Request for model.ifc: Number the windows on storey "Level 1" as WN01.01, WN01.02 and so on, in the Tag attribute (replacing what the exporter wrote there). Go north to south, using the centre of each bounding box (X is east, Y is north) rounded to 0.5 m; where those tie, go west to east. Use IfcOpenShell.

First a look at what the model holds.

```python
import ifcopenshell
import ifcopenshell.util.element
import ifcopenshell.util.placement

model = ifcopenshell.open("model.ifc")
print(model.schema)
storey = next(s for s in model.by_type("IfcBuildingStorey") if s.Name == "Level 1")
windows = [e for e in ifcopenshell.util.element.get_decomposition(storey) if e.is_a("IfcWindow")]
for e in sorted(windows, key=lambda e: e.id()):
    origin = ifcopenshell.util.placement.get_local_placement(e.ObjectPlacement)[:3, 3]
    print(e.id(), e.Tag, e.Name, origin.round(2) + 0.0, sep=" | ")
```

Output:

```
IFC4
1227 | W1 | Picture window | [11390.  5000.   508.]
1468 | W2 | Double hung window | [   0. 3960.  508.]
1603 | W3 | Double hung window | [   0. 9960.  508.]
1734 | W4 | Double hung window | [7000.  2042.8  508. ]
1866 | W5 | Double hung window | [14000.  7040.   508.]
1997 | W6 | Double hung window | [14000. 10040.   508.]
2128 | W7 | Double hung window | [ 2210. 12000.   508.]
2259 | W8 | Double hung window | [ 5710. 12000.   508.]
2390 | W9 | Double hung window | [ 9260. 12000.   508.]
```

```python
import ifcopenshell
import ifcopenshell.geom
import ifcopenshell.util.element
import ifcopenshell.util.shape

model = ifcopenshell.open("model.ifc")
settings = ifcopenshell.geom.settings()
settings.set("use-world-coords", True)


def centre(element):
    shape = ifcopenshell.geom.create_shape(settings, element)
    return ifcopenshell.util.shape.get_bbox_centroid(shape.geometry)


storey = next(s for s in model.by_type("IfcBuildingStorey") if s.Name == "Level 1")
windows = [e for e in ifcopenshell.util.element.get_decomposition(storey) if e.is_a("IfcWindow")]

# Insertion points can sit at a corner or the storey origin, so sort by the geometry (in metres).
centres = {e: centre(e) for e in windows}
windows.sort(key=lambda e: (-round(centres[e][1] / 0.5), centres[e][0]))

for i, e in enumerate(windows, start=1):
    number = f"WN01.{i:02d}"
    e.Tag = number
    print(e.id(), number)

model.write("model_updated.ifc")
```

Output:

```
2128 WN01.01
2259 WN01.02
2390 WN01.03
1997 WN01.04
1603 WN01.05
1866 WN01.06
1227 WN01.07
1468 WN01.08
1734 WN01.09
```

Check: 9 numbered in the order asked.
